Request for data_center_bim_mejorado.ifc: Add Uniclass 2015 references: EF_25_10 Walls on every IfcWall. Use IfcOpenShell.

First a look at what the model holds.

```python
import ifcopenshell

model = ifcopenshell.open("data_center_bim_mejorado.ifc")
print(model.schema)
print("classifications:", [c.Name for c in model.by_type("IfcClassification")])
for ifc_class in ("IfcDoor", "IfcRoof", "IfcStair", "IfcWall", "IfcWindow"):
    print(ifc_class, len(model.by_type(ifc_class)))
```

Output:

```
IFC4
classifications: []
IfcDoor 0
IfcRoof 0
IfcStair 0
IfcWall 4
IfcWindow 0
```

```python
import ifcopenshell
import ifcopenshell.api.classification

model = ifcopenshell.open("data_center_bim_mejorado.ifc")

system = ifcopenshell.api.classification.add_classification(model, classification="Uniclass 2015")

codes = {
    "IfcWall": ("EF_25_10", "Walls"),
}
for ifc_class, (code, name) in codes.items():
    products = model.by_type(ifc_class)
    ifcopenshell.api.classification.add_reference(
        model, products=products, classification=system, identification=code, name=name
    )
    print(code, len(products))

model.write("data_center_bim_mejorado_updated.ifc")
```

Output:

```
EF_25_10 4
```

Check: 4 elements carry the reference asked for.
